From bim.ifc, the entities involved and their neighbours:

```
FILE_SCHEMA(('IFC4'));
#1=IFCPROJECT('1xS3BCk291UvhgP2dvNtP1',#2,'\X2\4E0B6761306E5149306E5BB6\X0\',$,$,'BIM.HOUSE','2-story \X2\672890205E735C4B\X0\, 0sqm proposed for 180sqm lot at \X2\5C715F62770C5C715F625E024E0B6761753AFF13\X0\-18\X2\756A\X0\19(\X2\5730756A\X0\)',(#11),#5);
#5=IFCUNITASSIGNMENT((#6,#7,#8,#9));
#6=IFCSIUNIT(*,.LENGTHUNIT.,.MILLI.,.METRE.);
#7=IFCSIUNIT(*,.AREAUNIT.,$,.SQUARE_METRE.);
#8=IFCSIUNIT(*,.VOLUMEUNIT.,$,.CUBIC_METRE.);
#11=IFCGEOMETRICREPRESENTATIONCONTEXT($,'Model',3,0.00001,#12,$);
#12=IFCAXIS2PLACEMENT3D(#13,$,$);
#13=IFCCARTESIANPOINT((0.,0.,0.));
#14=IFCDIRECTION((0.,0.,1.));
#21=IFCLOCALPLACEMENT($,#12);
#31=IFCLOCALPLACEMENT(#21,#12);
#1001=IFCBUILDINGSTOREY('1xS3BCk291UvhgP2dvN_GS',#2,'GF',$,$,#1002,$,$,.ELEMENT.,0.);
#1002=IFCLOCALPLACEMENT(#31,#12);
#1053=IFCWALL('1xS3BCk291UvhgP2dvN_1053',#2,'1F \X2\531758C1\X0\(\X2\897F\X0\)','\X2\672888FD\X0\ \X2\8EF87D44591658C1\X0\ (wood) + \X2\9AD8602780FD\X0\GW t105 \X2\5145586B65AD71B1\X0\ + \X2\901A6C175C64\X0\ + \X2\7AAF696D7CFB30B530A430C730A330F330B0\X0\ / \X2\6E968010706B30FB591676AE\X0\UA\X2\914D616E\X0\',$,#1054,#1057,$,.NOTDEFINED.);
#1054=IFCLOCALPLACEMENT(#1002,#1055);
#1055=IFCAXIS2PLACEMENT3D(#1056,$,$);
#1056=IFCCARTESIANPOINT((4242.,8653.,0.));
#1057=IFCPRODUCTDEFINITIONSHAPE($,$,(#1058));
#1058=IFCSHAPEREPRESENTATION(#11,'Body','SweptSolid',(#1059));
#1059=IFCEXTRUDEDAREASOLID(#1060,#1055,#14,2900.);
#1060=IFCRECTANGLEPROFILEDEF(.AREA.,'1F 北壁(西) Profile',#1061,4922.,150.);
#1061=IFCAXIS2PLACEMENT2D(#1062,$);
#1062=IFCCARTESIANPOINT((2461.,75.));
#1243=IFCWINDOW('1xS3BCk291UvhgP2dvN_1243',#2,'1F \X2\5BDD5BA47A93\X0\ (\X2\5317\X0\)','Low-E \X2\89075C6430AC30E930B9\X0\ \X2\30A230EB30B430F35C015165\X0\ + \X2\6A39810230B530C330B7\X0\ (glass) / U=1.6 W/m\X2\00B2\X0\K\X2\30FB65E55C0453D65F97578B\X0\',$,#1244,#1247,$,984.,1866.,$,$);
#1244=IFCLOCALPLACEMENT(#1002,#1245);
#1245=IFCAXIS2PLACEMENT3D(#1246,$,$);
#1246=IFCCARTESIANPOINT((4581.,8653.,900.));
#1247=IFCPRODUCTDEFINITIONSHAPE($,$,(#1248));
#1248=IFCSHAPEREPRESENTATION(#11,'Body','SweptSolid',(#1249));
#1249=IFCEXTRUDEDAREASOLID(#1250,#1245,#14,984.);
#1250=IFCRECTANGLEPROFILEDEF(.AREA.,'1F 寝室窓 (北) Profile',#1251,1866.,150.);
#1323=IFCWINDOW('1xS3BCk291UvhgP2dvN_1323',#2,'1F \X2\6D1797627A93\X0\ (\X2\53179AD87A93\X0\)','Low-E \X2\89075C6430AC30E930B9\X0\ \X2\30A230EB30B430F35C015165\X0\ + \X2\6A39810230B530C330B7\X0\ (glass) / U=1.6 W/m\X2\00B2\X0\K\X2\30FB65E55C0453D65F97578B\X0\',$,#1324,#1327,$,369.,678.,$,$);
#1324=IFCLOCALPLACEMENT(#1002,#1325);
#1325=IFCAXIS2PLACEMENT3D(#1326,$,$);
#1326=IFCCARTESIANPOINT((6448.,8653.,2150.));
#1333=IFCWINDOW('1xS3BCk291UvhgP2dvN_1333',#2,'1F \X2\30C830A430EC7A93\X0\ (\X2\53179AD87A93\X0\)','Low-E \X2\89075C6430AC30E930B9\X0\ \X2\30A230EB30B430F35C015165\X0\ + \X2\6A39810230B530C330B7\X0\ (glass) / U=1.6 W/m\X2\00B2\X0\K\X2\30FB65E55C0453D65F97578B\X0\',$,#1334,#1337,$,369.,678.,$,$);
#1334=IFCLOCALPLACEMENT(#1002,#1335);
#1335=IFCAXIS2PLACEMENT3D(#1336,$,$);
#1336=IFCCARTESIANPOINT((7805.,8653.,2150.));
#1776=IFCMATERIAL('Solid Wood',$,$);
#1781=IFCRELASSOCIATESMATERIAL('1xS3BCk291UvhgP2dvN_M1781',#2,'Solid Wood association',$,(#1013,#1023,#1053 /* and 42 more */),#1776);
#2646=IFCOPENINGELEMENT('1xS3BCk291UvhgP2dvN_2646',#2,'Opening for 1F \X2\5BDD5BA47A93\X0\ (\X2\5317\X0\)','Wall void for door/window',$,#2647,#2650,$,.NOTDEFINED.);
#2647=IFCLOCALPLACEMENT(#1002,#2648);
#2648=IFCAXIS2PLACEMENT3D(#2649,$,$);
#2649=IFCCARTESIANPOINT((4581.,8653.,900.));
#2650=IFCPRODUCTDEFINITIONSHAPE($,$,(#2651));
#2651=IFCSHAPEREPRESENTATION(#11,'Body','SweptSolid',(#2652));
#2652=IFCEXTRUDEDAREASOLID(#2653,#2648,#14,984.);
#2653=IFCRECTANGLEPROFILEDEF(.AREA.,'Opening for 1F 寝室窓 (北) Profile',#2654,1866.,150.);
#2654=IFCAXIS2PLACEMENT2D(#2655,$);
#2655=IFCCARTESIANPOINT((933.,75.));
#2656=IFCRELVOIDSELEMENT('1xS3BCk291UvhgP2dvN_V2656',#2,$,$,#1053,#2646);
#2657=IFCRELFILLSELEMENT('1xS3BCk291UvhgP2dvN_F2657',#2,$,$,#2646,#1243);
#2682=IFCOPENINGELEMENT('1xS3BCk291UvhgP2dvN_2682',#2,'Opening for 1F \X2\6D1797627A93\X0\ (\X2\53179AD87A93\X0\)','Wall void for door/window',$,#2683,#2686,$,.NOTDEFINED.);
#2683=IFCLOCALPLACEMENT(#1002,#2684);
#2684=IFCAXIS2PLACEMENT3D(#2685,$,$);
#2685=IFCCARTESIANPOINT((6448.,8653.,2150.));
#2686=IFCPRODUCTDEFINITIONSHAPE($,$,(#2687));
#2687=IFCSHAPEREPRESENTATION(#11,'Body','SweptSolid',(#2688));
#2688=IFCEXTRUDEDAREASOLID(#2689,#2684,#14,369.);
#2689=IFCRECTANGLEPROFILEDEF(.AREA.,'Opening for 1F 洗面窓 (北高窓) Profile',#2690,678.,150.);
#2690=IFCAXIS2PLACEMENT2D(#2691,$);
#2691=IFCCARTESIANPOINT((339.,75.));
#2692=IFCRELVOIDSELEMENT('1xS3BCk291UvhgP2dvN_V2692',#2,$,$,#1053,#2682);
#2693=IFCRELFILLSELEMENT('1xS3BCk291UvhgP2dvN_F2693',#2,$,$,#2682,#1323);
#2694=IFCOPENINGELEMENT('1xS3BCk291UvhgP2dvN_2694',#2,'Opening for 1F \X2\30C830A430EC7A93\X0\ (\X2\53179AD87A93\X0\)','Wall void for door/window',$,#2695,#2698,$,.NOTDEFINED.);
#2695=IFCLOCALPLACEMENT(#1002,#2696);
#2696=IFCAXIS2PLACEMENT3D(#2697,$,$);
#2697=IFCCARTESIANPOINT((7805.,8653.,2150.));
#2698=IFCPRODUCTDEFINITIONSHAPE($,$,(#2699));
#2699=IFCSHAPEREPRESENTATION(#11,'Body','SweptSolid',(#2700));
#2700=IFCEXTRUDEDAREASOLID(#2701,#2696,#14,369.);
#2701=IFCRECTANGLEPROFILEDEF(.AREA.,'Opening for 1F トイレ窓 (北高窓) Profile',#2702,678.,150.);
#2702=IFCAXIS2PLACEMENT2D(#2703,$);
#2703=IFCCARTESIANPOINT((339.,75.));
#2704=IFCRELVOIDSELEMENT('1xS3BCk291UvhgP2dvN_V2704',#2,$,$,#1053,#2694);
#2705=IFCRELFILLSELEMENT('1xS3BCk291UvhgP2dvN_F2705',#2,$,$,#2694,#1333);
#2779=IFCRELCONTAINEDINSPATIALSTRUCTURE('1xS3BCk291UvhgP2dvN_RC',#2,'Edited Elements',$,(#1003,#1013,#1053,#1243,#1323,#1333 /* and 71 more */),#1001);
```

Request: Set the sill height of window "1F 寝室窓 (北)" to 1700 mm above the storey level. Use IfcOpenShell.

```python
import numpy as np
import ifcopenshell
import ifcopenshell.api.geometry
import ifcopenshell.geom
import ifcopenshell.util.element
import ifcopenshell.util.placement
import ifcopenshell.util.shape
import ifcopenshell.util.unit

model = ifcopenshell.open("bim.ifc")
unit_scale = ifcopenshell.util.unit.calculate_unit_scale(model)

window = model.by_id(1243)
opening = window.FillsVoids[0].RelatingOpeningElement
storey = ifcopenshell.util.element.get_container(window, ifc_class="IfcBuildingStorey")
level = ifcopenshell.util.placement.get_local_placement(storey.ObjectPlacement)[2, 3]

# The opening's origin need not be at the sill, so measure its lowest point.
shape = ifcopenshell.geom.create_shape(ifcopenshell.geom.settings(), opening)
bottom = ifcopenshell.util.shape.get_shape_bottom_elevation(shape, shape.geometry) / unit_scale
dz = level + 1.7 / unit_scale - bottom

shift = np.array([0.0, 0.0, dz])
# The window is not placed relative to its opening, so move both.
for product in (opening, window):
    matrix = ifcopenshell.util.placement.get_local_placement(product.ObjectPlacement)
    matrix[:3, 3] += shift
    ifcopenshell.api.geometry.edit_object_placement(model, product=product, matrix=matrix, is_si=False)

print(f"moved by {dz * unit_scale:+.3f} m")

model.write("bim-out.ifc")
```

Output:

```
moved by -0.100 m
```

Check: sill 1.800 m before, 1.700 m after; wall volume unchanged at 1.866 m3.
